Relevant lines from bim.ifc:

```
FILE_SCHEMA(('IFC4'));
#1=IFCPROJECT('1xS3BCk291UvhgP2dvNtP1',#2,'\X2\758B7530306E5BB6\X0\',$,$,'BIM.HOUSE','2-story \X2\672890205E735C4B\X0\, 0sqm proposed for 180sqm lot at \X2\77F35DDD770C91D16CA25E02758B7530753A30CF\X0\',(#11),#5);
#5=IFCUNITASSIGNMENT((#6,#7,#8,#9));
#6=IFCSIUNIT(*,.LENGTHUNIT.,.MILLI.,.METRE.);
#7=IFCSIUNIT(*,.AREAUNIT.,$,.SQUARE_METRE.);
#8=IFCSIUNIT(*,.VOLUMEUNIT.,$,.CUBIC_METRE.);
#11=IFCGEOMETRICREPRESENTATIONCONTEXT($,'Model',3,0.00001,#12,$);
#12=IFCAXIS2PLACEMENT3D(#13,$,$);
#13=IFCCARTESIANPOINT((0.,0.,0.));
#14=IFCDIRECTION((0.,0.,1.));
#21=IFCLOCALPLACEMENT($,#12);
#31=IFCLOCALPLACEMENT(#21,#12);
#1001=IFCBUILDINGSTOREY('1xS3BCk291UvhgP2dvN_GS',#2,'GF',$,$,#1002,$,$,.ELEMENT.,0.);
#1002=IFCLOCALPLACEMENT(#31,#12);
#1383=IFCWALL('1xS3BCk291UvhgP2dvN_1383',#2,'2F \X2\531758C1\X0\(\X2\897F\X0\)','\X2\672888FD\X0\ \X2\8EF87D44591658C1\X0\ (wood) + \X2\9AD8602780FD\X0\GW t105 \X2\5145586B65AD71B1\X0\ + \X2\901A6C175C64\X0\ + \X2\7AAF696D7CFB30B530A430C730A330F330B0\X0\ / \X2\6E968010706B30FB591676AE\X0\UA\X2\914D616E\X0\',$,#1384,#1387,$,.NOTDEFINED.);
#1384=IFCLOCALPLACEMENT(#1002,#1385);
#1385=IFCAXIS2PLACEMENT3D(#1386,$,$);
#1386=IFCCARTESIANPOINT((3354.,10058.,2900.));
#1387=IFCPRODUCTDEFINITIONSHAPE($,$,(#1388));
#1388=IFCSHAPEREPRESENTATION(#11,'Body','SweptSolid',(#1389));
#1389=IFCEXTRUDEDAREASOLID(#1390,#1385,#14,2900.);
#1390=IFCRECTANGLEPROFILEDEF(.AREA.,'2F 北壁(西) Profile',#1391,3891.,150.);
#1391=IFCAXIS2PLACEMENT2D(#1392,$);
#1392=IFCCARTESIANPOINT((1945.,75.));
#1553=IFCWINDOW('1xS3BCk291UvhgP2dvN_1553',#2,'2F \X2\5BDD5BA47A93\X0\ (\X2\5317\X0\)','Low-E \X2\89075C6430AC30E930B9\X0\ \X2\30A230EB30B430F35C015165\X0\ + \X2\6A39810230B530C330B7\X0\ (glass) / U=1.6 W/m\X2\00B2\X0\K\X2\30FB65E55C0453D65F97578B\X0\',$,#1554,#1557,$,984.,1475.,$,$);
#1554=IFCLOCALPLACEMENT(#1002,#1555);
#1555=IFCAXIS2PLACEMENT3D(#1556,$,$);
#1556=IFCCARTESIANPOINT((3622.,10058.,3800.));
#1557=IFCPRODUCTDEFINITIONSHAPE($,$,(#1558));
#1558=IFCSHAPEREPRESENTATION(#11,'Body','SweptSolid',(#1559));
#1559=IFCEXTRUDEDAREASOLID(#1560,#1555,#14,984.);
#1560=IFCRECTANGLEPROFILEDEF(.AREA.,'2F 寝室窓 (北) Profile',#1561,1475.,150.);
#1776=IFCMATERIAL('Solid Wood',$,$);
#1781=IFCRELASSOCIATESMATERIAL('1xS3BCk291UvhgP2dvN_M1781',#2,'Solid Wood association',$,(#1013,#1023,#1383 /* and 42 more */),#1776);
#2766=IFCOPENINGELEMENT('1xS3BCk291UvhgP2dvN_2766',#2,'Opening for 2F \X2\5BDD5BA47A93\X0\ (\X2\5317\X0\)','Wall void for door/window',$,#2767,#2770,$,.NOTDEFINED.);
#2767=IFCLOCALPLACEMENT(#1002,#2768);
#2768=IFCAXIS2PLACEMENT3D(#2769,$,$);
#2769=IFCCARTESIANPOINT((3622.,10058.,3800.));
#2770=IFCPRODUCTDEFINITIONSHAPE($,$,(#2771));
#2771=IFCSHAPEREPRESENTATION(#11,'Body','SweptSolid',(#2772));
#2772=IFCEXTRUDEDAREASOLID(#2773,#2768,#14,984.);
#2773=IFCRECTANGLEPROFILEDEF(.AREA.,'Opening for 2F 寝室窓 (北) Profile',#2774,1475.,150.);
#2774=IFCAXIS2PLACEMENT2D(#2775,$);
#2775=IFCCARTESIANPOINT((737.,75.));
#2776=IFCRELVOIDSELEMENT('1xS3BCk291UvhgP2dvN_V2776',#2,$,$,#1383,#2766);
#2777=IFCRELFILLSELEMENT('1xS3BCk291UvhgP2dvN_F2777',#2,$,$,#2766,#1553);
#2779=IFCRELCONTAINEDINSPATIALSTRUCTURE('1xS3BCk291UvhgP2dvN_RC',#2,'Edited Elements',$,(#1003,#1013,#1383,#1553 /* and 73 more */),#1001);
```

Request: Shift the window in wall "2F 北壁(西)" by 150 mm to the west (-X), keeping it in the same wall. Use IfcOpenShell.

```python
import ifcopenshell
import ifcopenshell.api.geometry
import ifcopenshell.util.placement

model = ifcopenshell.open("bim.ifc")

window = model.by_guid("1xS3BCk291UvhgP2dvN_1553")
opening = window.FillsVoids[0].RelatingOpeningElement
wall = opening.VoidsElements[0].RelatingBuildingElement

wall_matrix = ifcopenshell.util.placement.get_local_placement(wall.ObjectPlacement)
shift = wall_matrix[:3, 0] * -150.0
before = ifcopenshell.util.placement.get_local_placement(window.ObjectPlacement)[:3, 3].copy()

# The window is not placed relative to its opening, so move both.
for product in (opening, window):
    matrix = ifcopenshell.util.placement.get_local_placement(product.ObjectPlacement)
    matrix[:3, 3] += shift
    ifcopenshell.api.geometry.edit_object_placement(model, product=product, matrix=matrix, is_si=False)

after = ifcopenshell.util.placement.get_local_placement(window.ObjectPlacement)[:3, 3]
print("window moved by", (after - before).round(3) + 0.0)

model.write("bim_updated.ifc")
```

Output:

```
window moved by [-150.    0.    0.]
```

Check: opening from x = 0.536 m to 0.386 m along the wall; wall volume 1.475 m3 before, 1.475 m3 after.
